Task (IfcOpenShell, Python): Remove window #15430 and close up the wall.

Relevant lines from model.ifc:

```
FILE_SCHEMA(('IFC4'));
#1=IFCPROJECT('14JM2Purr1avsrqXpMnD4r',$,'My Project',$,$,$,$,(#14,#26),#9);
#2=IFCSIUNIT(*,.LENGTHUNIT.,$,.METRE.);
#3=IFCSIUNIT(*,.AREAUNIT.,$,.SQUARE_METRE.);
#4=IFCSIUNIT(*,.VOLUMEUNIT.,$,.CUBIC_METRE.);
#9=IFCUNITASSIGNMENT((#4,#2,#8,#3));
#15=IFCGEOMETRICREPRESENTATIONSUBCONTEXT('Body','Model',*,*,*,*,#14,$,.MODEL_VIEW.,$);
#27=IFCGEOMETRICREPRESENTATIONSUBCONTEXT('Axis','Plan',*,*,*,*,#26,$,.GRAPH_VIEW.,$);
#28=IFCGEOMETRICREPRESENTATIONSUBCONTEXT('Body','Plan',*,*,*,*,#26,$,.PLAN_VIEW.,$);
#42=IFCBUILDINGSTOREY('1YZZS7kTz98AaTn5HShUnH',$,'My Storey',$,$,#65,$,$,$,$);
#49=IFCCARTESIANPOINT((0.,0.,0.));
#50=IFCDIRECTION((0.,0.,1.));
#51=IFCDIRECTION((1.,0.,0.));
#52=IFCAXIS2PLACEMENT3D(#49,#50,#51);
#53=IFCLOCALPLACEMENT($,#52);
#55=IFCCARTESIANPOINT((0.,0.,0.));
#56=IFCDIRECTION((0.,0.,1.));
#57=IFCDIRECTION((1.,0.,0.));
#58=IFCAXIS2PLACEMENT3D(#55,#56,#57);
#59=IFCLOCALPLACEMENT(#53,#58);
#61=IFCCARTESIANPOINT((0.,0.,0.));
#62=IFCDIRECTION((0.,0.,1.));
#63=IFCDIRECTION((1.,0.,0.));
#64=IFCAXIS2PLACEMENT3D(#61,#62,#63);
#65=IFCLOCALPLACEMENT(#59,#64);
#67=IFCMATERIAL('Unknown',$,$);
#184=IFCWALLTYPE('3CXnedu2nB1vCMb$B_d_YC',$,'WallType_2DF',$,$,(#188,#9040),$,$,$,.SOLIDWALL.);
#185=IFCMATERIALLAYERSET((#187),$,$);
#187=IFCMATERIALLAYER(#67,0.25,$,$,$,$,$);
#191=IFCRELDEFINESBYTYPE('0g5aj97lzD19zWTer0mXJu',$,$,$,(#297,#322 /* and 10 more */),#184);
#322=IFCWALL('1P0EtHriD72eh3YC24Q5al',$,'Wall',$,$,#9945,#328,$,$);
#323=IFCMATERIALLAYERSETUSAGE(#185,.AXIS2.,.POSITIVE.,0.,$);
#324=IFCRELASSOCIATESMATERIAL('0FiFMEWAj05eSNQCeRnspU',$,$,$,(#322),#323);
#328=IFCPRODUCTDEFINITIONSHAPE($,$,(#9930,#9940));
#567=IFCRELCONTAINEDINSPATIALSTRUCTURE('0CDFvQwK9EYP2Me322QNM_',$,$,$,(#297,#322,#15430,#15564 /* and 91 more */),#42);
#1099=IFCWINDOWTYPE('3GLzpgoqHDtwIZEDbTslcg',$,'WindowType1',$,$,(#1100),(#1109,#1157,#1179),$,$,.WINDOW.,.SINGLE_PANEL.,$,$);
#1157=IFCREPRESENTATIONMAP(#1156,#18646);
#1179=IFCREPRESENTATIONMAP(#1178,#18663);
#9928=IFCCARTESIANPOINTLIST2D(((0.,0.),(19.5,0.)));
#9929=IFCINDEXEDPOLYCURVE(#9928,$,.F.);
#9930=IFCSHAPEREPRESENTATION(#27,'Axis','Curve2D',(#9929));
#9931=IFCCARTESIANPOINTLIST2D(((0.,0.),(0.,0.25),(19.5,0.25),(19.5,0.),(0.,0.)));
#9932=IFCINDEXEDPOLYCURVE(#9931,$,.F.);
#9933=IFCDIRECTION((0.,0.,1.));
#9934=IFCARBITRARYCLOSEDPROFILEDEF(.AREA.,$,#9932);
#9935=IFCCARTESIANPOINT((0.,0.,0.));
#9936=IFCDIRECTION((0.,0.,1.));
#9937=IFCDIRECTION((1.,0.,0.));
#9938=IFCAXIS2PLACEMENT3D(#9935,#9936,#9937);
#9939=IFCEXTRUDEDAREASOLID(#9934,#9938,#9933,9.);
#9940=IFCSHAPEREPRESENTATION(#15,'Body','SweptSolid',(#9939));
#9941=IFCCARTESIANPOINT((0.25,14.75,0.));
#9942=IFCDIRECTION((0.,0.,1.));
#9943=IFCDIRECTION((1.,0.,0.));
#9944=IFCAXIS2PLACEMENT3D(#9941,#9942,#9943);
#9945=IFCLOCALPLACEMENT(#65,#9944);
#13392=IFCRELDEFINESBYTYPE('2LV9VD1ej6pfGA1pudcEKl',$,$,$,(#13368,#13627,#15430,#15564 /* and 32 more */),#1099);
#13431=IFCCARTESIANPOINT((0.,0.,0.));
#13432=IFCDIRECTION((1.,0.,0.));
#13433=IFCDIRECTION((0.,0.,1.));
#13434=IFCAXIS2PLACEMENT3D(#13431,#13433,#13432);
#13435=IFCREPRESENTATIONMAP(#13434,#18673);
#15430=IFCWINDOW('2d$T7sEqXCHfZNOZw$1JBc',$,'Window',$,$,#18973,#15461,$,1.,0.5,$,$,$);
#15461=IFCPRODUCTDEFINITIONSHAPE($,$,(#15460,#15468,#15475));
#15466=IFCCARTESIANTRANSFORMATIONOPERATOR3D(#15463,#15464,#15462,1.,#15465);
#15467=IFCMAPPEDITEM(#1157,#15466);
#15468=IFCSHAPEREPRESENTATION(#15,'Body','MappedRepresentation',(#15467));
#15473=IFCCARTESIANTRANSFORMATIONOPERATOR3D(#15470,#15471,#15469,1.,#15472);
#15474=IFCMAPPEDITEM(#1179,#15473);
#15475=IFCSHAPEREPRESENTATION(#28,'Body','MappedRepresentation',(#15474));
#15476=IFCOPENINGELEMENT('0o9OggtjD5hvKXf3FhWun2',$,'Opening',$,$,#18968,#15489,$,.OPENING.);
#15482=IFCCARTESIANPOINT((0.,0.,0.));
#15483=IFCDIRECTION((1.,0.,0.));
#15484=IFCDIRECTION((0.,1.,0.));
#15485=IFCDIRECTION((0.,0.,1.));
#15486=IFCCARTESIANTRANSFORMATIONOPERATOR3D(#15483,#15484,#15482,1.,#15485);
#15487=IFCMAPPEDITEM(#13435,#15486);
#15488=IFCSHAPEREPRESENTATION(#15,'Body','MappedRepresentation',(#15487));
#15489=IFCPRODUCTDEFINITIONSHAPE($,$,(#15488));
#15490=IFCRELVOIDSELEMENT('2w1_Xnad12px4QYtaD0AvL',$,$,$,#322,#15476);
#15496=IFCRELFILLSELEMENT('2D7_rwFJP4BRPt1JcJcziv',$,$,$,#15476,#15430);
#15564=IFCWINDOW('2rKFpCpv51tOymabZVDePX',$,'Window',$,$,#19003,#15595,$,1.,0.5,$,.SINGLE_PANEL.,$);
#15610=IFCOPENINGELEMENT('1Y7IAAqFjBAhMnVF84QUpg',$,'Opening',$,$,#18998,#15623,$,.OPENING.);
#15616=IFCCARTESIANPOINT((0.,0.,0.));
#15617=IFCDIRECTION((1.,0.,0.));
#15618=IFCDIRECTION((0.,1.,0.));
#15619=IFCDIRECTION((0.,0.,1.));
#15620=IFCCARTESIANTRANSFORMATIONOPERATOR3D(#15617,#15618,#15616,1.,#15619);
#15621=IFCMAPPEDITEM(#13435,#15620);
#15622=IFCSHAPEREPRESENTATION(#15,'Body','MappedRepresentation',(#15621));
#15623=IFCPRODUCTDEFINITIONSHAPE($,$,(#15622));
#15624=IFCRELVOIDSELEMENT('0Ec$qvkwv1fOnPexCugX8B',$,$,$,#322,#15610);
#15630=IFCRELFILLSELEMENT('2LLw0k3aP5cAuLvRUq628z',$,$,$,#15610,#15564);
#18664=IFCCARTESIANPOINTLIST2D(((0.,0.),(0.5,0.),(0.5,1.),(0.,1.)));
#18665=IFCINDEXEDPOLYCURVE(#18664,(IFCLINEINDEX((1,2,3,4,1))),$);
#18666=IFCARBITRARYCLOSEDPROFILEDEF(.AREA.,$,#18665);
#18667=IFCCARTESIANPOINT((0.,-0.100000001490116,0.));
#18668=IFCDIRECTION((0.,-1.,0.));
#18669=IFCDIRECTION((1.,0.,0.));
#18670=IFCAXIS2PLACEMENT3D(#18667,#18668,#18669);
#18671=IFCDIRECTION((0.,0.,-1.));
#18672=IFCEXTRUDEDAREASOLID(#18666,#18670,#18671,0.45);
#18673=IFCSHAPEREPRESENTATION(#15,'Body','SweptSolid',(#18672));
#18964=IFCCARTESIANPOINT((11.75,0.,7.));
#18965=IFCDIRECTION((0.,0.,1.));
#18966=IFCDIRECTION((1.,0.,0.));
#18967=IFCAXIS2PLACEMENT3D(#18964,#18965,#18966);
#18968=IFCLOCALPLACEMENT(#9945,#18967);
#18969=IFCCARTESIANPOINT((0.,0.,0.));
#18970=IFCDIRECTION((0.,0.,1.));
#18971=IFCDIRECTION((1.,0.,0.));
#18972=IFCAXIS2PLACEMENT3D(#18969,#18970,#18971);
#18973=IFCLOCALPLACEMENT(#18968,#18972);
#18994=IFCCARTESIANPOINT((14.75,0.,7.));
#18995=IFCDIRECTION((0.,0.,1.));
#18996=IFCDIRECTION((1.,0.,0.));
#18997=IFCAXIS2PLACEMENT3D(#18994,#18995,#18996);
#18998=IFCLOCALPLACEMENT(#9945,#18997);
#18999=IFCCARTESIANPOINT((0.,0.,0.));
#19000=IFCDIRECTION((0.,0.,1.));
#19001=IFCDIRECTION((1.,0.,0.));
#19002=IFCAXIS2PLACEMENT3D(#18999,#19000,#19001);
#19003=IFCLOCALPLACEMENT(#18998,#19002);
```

```python
import ifcopenshell
import ifcopenshell.api.feature
import ifcopenshell.api.root
import ifcopenshell.geom
import ifcopenshell.util.shape

model = ifcopenshell.open("model.ifc")
settings = ifcopenshell.geom.settings()


def volume(element):
    """Net volume in cubic metres, openings subtracted."""
    shape = ifcopenshell.geom.create_shape(settings, element)
    return ifcopenshell.util.shape.get_volume(shape.geometry)


window = model.by_id(15430)
opening = window.FillsVoids[0].RelatingOpeningElement
wall = opening.VoidsElements[0].RelatingBuildingElement
before = volume(wall)

ifcopenshell.api.root.remove_product(model, product=window)
ifcopenshell.api.feature.remove_feature(model, feature=opening)

after = volume(wall)

print(f"wall volume {before:.3f} -> {after:.3f} m3")

model.write("model-out.ifc")
```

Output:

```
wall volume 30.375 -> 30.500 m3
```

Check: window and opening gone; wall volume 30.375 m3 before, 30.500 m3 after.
